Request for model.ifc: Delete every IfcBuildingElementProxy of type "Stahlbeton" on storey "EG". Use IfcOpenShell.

First a look at what the model holds.

```python
import ifcopenshell
import ifcopenshell.util.element

model = ifcopenshell.open("model.ifc")
print(model.schema)
storey = next(s for s in model.by_type("IfcBuildingStorey") if s.Name == "EG")
proxies = [e for e in ifcopenshell.util.element.get_decomposition(storey) if e.is_a("IfcBuildingElementProxy")]
seen = {}
for e in proxies:
    element_type = ifcopenshell.util.element.get_type(e)
    name = element_type.Name if element_type not in (None, e) else None
    seen[name] = seen.get(name, 0) + 1
for name, count in sorted(seen.items(), key=str):
    print(count, "x", name)
```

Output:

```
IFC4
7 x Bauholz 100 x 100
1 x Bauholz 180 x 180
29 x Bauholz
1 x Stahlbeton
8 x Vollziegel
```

```python
import ifcopenshell
import ifcopenshell.api.root
import ifcopenshell.util.element

model = ifcopenshell.open("model.ifc")

storey = next(s for s in model.by_type("IfcBuildingStorey") if s.Name == "EG")
proxies = [e for e in ifcopenshell.util.element.get_decomposition(storey) if e.is_a("IfcBuildingElementProxy")]
targets = [e for e in proxies if (t := ifcopenshell.util.element.get_type(e)) not in (None, e) and t.Name == "Stahlbeton"]

for e in targets:
    ifcopenshell.api.root.remove_product(model, product=e)
print(len(targets), "removed")

model.write("model_v2.ifc")
```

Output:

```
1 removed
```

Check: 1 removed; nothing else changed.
